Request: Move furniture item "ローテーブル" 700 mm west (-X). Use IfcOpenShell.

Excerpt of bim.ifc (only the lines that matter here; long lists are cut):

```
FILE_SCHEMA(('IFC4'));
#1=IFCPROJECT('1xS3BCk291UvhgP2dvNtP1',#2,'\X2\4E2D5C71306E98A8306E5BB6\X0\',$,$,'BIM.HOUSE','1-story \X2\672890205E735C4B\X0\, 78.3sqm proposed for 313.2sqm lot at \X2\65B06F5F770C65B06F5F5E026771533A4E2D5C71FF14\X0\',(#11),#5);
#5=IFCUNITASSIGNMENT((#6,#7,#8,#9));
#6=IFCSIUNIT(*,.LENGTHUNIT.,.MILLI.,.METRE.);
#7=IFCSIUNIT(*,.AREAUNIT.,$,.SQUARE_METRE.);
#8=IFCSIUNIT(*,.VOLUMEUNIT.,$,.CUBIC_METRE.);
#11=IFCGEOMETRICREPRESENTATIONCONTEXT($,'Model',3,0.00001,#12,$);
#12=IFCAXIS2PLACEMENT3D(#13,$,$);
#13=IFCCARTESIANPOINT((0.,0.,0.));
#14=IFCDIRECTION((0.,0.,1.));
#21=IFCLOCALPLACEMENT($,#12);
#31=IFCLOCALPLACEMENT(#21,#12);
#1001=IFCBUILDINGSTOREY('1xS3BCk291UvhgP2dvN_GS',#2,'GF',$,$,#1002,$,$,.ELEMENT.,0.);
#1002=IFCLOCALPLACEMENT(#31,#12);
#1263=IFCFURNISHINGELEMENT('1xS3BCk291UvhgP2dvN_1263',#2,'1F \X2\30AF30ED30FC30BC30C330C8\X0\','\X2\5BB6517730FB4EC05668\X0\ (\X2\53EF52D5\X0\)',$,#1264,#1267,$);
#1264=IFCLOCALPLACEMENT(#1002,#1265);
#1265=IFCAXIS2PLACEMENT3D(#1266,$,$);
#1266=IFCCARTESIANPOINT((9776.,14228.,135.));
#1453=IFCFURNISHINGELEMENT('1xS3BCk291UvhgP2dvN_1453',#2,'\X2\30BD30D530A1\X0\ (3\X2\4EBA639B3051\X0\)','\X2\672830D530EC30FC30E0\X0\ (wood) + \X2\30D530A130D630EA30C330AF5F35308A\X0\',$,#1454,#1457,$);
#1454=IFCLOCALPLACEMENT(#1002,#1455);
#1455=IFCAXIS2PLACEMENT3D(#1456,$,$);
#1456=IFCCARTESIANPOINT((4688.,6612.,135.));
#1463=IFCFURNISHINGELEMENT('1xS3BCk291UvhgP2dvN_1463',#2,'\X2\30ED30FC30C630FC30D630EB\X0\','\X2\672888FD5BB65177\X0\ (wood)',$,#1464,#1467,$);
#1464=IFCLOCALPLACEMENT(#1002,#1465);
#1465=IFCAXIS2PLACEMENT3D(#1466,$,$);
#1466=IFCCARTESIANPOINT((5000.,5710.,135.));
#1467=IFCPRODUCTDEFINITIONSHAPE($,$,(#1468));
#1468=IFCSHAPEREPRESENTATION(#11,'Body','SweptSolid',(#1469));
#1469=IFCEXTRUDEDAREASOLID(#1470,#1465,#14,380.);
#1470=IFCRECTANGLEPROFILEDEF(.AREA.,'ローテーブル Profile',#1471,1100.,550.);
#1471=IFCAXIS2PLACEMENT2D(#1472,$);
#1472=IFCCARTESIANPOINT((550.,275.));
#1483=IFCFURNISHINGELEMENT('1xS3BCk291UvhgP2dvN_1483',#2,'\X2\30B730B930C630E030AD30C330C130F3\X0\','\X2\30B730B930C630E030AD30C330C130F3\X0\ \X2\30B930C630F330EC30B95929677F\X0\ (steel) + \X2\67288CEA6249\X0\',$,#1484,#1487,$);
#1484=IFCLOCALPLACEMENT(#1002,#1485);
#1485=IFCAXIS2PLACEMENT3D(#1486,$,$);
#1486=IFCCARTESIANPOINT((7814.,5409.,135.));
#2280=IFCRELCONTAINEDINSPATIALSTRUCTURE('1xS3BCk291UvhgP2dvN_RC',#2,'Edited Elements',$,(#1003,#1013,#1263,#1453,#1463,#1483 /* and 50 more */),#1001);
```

```python
import ifcopenshell
import ifcopenshell.api.geometry
import ifcopenshell.util.placement
import ifcopenshell.util.unit

model = ifcopenshell.open("bim.ifc")
unit_scale = ifcopenshell.util.unit.calculate_unit_scale(model)

item = model.by_guid("1xS3BCk291UvhgP2dvN_1463")
matrix = ifcopenshell.util.placement.get_local_placement(item.ObjectPlacement)
matrix[0, 3] -= 0.7 / unit_scale
ifcopenshell.api.geometry.edit_object_placement(model, product=item, matrix=matrix, is_si=False)

print(ifcopenshell.util.placement.get_local_placement(item.ObjectPlacement).round(3) + 0.0)

model.write("bim_edited.ifc")
```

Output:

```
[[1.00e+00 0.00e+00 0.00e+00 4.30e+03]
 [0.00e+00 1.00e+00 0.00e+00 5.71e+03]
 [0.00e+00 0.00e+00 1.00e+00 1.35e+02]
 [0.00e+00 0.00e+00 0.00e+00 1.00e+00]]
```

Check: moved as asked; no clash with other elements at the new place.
